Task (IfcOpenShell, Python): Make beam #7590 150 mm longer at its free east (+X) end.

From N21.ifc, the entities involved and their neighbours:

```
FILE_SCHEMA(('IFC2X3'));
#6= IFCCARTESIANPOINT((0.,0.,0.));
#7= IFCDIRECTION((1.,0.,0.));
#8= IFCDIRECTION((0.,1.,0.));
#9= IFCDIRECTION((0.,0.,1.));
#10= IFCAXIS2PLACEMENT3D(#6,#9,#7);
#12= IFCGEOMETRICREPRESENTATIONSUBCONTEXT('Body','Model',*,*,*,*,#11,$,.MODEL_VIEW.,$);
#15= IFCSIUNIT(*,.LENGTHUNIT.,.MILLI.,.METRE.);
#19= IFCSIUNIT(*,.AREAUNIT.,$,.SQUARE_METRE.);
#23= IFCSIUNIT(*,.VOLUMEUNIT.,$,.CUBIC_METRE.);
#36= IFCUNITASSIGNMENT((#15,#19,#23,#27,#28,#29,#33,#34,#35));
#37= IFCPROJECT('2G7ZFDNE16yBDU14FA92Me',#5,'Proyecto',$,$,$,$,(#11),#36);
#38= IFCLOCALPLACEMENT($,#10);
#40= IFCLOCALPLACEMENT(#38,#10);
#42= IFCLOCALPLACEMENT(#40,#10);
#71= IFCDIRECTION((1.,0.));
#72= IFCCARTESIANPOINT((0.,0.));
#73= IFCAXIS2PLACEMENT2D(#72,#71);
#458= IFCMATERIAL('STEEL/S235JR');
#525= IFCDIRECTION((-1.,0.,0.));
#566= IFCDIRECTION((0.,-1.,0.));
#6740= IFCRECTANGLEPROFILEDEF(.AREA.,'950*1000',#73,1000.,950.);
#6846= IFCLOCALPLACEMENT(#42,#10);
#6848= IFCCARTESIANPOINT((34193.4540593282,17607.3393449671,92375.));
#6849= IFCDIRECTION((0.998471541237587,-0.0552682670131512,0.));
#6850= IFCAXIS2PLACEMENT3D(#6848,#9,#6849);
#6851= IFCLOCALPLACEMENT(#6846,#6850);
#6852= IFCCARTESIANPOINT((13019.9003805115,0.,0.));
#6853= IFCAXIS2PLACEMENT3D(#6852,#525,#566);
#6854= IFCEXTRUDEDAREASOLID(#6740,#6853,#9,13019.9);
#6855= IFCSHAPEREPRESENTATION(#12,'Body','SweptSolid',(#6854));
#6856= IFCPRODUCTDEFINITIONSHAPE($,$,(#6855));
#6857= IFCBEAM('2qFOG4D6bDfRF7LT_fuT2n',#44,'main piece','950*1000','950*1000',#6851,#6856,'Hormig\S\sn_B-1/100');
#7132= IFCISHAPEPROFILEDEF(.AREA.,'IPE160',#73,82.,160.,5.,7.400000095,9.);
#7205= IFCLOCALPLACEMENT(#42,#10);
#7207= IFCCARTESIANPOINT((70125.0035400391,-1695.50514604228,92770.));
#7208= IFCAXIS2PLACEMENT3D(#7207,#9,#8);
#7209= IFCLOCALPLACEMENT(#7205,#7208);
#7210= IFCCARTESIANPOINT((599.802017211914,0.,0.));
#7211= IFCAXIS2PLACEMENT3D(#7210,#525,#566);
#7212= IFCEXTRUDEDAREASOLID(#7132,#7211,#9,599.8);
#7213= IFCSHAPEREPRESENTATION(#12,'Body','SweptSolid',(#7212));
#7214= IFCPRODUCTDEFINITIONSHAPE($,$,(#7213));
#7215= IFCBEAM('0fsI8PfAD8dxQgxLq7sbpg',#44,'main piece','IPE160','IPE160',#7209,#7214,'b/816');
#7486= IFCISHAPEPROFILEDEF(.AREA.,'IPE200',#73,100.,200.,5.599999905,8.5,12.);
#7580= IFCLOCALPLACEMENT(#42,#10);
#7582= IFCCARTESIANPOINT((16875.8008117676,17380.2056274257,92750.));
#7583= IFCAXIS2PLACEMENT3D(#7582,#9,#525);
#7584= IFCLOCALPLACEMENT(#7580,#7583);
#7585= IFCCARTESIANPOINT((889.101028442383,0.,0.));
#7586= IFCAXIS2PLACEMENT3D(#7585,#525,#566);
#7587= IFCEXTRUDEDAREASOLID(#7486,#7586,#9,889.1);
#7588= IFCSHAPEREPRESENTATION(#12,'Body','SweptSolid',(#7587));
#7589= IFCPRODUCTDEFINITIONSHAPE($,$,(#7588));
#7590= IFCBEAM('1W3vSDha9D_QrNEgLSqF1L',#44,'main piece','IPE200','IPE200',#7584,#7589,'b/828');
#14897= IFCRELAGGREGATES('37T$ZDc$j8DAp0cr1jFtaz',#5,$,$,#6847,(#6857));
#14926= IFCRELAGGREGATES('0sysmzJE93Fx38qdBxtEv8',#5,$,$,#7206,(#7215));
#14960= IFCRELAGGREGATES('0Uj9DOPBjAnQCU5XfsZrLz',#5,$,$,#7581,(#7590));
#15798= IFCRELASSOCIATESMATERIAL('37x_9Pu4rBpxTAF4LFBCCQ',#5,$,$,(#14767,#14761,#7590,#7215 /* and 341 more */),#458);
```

```python
import ifcopenshell
import ifcopenshell.util.representation
import ifcopenshell.util.unit

model = ifcopenshell.open("N21.ifc")
unit_scale = ifcopenshell.util.unit.calculate_unit_scale(model)

member = model.by_guid("1W3vSDha9D_QrNEgLSqF1L")
change = 0.15 / unit_scale

# The extrusion runs towards the end named, so only its depth changes.
body = ifcopenshell.util.representation.get_representation(member, "Model", "Body")
solid = body.Items[0]
old_length = solid.Depth
solid.Depth += change

print(f"length {old_length:g} -> {solid.Depth:g}")

model.write("N21_rev.ifc")
```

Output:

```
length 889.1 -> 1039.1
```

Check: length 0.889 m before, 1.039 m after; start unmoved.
